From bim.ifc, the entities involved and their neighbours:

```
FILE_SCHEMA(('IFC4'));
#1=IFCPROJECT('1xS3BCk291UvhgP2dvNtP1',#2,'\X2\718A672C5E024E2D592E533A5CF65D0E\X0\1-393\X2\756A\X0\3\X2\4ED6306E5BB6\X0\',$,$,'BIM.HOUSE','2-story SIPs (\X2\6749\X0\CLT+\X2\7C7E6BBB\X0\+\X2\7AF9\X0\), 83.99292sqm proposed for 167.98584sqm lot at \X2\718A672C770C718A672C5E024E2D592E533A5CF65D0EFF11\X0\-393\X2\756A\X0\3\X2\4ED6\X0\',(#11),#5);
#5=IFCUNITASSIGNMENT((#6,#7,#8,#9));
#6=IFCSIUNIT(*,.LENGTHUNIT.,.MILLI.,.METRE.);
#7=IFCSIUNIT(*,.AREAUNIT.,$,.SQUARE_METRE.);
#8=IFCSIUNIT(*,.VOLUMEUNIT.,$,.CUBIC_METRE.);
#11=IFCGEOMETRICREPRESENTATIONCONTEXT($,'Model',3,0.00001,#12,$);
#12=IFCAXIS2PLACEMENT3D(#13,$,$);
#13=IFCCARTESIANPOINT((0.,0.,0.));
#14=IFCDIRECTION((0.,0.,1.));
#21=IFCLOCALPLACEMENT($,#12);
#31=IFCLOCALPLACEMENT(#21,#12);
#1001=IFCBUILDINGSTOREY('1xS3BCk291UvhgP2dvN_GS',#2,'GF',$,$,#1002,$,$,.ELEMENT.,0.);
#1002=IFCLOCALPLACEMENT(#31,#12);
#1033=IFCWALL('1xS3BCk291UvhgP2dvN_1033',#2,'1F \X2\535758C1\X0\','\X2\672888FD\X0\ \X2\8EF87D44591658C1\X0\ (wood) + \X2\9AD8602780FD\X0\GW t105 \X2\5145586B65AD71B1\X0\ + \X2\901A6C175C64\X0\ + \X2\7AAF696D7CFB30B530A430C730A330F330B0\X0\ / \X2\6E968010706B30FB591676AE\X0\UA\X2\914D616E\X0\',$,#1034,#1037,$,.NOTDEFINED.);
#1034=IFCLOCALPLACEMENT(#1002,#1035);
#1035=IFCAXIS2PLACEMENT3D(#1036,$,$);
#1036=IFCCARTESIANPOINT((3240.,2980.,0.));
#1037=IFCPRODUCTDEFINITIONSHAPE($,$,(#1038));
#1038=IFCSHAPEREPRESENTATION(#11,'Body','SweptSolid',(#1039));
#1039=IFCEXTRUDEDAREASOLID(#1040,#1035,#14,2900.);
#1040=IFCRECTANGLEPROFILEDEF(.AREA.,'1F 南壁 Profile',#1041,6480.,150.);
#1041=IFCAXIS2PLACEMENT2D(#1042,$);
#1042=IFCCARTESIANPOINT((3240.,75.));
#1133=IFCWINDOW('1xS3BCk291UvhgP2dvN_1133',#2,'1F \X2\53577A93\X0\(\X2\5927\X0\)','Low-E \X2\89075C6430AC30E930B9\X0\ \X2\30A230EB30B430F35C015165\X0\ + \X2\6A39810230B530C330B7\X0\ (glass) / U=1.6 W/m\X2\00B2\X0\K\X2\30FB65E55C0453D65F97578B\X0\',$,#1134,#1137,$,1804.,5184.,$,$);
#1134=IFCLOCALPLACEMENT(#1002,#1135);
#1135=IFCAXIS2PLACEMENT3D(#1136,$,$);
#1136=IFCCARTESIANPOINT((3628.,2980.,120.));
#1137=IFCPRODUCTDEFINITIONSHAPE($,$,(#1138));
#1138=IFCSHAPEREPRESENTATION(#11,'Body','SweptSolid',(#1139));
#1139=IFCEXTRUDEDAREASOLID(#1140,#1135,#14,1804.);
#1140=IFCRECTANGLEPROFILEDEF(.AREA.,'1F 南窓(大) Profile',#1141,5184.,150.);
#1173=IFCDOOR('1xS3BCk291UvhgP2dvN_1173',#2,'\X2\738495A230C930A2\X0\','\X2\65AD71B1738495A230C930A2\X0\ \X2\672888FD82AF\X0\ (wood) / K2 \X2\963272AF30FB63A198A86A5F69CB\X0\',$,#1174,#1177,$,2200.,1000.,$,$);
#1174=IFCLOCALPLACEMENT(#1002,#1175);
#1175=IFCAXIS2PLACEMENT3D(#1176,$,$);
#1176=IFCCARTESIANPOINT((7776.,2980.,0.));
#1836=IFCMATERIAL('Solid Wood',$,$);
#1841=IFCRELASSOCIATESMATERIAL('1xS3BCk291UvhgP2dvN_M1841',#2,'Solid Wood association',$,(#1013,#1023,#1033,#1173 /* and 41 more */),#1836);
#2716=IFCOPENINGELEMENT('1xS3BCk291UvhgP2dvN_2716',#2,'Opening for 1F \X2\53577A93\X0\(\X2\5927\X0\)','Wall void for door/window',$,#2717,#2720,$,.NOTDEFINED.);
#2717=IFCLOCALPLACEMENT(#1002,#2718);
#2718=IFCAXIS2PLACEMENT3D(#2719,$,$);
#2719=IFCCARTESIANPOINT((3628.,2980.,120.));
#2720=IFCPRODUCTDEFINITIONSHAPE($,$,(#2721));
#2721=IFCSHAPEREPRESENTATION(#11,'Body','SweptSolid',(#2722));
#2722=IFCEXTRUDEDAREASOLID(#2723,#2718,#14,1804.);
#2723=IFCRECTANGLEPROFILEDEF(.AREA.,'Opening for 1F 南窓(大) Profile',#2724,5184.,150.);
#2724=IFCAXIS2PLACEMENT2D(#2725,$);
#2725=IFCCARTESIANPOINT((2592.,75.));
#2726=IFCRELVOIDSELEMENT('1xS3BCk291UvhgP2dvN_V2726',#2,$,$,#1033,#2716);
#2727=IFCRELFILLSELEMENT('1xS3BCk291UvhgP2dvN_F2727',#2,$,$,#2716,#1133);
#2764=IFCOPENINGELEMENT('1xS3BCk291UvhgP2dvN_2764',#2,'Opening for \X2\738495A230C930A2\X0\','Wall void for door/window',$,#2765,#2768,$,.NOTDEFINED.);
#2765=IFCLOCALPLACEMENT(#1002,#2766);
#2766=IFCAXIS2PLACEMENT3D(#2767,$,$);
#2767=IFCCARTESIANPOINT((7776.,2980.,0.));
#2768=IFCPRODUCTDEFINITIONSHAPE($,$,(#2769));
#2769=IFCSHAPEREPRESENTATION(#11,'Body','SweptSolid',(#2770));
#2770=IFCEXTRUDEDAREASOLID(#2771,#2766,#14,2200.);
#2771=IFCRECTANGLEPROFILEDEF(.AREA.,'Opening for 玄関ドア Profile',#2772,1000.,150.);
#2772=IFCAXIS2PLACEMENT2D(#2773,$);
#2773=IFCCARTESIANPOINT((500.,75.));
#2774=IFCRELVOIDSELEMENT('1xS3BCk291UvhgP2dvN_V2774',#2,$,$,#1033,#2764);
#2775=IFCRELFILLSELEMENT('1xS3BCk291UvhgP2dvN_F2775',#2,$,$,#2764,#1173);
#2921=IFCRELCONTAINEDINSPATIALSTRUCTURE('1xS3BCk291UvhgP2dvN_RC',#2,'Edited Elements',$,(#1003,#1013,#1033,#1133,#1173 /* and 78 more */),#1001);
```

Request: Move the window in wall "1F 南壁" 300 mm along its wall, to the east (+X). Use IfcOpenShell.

```python
import ifcopenshell
import ifcopenshell.api.geometry
import ifcopenshell.util.placement

model = ifcopenshell.open("bim.ifc")

window = model.by_guid("1xS3BCk291UvhgP2dvN_1133")
opening = window.FillsVoids[0].RelatingOpeningElement
wall = opening.VoidsElements[0].RelatingBuildingElement

wall_matrix = ifcopenshell.util.placement.get_local_placement(wall.ObjectPlacement)
shift = wall_matrix[:3, 0] * 300.0
before = ifcopenshell.util.placement.get_local_placement(window.ObjectPlacement)[:3, 3].copy()

# The window is not placed relative to its opening, so move both.
for product in (opening, window):
    matrix = ifcopenshell.util.placement.get_local_placement(product.ObjectPlacement)
    matrix[:3, 3] += shift
    ifcopenshell.api.geometry.edit_object_placement(model, product=product, matrix=matrix, is_si=False)

after = ifcopenshell.util.placement.get_local_placement(window.ObjectPlacement)[:3, 3]
print("window moved by", (after - before).round(3) + 0.0)

model.write("bim-out.ifc")
```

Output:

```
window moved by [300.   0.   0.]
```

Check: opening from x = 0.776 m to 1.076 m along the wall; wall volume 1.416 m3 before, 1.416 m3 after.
